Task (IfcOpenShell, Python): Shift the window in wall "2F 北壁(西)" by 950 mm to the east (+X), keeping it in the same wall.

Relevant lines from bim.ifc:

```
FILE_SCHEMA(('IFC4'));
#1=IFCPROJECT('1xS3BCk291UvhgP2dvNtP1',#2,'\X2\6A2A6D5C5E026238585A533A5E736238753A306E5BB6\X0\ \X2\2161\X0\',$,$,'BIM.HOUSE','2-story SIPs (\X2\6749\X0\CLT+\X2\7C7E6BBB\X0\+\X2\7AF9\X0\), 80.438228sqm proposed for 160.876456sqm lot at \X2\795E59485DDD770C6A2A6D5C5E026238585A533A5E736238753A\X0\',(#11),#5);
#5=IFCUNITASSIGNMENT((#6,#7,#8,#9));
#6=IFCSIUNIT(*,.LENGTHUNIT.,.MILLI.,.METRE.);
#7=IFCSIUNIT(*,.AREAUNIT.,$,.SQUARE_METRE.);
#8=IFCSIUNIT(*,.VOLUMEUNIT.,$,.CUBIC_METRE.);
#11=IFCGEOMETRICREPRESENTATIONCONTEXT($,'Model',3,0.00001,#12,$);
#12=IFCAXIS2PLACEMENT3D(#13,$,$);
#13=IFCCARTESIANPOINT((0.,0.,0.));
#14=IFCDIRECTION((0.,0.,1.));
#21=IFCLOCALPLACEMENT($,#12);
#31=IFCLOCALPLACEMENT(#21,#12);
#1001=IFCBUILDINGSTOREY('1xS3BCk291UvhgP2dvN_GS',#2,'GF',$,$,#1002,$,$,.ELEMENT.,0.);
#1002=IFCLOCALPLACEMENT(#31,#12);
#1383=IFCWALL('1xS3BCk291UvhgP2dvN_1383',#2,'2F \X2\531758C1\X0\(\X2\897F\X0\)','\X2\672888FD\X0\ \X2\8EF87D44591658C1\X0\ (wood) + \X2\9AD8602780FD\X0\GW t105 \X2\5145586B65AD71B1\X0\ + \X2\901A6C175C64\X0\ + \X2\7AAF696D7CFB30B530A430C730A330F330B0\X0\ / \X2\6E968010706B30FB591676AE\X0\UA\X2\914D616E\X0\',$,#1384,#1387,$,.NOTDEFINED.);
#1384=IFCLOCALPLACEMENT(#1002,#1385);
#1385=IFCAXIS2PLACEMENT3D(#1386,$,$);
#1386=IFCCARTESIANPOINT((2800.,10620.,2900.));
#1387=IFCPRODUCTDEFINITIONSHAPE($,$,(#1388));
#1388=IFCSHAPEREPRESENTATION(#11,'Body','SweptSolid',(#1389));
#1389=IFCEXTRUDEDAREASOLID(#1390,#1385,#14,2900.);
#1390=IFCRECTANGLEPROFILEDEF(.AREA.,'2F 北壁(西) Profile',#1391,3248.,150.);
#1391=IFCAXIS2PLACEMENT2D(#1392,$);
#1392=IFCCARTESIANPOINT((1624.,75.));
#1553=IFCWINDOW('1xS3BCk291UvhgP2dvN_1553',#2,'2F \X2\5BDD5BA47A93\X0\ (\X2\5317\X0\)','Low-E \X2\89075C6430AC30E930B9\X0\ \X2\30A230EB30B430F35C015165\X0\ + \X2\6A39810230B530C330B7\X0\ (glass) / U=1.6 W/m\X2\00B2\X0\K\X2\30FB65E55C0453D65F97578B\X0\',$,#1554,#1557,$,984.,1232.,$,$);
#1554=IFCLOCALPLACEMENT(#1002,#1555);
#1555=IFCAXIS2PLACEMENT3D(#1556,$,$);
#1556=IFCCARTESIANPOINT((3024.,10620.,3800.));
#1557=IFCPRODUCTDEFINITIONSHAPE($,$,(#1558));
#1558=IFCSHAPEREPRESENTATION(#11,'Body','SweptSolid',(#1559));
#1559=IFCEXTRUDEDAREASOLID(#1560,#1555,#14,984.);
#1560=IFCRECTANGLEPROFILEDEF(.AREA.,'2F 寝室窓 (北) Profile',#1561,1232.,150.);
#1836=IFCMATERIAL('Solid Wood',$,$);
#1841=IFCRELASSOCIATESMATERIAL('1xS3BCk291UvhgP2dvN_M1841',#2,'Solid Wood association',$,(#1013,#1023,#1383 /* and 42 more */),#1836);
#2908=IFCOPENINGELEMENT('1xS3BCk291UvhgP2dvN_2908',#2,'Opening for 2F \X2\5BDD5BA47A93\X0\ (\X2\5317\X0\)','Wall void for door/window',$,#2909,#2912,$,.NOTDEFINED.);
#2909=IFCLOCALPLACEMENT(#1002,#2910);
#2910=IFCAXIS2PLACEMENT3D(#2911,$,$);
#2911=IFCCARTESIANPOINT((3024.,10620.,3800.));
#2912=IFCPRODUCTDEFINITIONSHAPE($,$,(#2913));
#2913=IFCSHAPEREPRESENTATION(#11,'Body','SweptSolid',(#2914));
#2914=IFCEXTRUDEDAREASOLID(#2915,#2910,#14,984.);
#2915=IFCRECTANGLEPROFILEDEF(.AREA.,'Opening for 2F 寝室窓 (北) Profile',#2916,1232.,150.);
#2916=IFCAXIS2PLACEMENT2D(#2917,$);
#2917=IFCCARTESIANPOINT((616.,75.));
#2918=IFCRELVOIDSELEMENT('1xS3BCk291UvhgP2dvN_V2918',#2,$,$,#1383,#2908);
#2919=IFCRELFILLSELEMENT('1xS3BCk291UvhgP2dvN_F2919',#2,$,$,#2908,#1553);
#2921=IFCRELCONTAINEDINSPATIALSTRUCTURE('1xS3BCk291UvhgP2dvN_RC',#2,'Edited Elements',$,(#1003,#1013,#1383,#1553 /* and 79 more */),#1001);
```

```python
import ifcopenshell
import ifcopenshell.api.geometry
import ifcopenshell.util.placement

model = ifcopenshell.open("bim.ifc")

window = model.by_guid("1xS3BCk291UvhgP2dvN_1553")
opening = window.FillsVoids[0].RelatingOpeningElement
wall = opening.VoidsElements[0].RelatingBuildingElement

wall_matrix = ifcopenshell.util.placement.get_local_placement(wall.ObjectPlacement)
shift = wall_matrix[:3, 0] * 950.0
before = ifcopenshell.util.placement.get_local_placement(window.ObjectPlacement)[:3, 3].copy()

# The window is not placed relative to its opening, so move both.
for product in (opening, window):
    matrix = ifcopenshell.util.placement.get_local_placement(product.ObjectPlacement)
    matrix[:3, 3] += shift
    ifcopenshell.api.geometry.edit_object_placement(model, product=product, matrix=matrix, is_si=False)

after = ifcopenshell.util.placement.get_local_placement(window.ObjectPlacement)[:3, 3]
print("window moved by", (after - before).round(3) + 0.0)

model.write("bim-out.ifc")
```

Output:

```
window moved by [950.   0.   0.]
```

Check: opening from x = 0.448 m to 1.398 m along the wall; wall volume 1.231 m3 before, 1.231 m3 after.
